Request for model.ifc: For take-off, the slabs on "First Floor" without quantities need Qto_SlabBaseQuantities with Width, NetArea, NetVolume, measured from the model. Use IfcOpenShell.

First a look at what the model holds.

```python
import ifcopenshell
import ifcopenshell.util.element
import ifcopenshell.util.unit

model = ifcopenshell.open("model.ifc")
print(model.schema)
for unit_type in ("LENGTHUNIT", "AREAUNIT", "VOLUMEUNIT"):
    print(unit_type, ifcopenshell.util.unit.calculate_unit_scale(model, unit_type))
storey = next(s for s in model.by_type("IfcBuildingStorey") if s.Name == "First Floor")
slabs = [e for e in ifcopenshell.util.element.get_decomposition(storey) if e.is_a("IfcSlab")]
for e in sorted(slabs, key=lambda e: e.id()):
    print(e.id(), e.is_a(), e.Name, list(ifcopenshell.util.element.get_psets(e, qtos_only=True)), sep=" | ")
```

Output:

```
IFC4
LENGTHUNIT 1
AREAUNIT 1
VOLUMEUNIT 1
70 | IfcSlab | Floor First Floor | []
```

```python
import ifcopenshell
import ifcopenshell.api.pset
import ifcopenshell.geom
import ifcopenshell.util.element
import ifcopenshell.util.shape
import ifcopenshell.util.unit

model = ifcopenshell.open("model.ifc")
unit_scale = ifcopenshell.util.unit.calculate_unit_scale(model)
area_scale = ifcopenshell.util.unit.calculate_unit_scale(model, "AREAUNIT")
volume_scale = ifcopenshell.util.unit.calculate_unit_scale(model, "VOLUMEUNIT")
settings = ifcopenshell.geom.settings()

storey = next(s for s in model.by_type("IfcBuildingStorey") if s.Name == "First Floor")
slabs = [e for e in ifcopenshell.util.element.get_decomposition(storey) if e.is_a("IfcSlab")]

for e in sorted(slabs, key=lambda e: e.id()):
    if ifcopenshell.util.element.get_psets(e, qtos_only=True, should_inherit=False):
        continue
    # Geometry comes back in metres, in the element's own axes.
    shape = ifcopenshell.geom.create_shape(settings, e)
    values = {
        "Width": ifcopenshell.util.shape.get_z(shape.geometry) / unit_scale,
        "NetArea": ifcopenshell.util.shape.get_footprint_area(shape.geometry) / area_scale,
        "NetVolume": ifcopenshell.util.shape.get_volume(shape.geometry) / volume_scale,
    }
    qto = ifcopenshell.api.pset.add_qto(model, product=e, name="Qto_SlabBaseQuantities")
    ifcopenshell.api.pset.edit_qto(model, qto=qto, properties=values)
    print(e.id(), {k: round(v, 3) for k, v in values.items()})

model.write("model_updated.ifc")
```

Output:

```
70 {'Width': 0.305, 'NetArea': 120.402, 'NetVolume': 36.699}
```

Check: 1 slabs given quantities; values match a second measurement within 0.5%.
